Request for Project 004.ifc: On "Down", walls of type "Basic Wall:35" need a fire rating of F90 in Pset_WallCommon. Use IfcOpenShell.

First a look at what the model holds.

```python
import ifcopenshell
import ifcopenshell.util.element

model = ifcopenshell.open("Project 004.ifc")
print(model.schema)
storey = next(s for s in model.by_type("IfcBuildingStorey") if s.Name == "Down")
walls = [e for e in ifcopenshell.util.element.get_decomposition(storey) if e.is_a("IfcWall")]
seen = {}
for e in walls:
    element_type = ifcopenshell.util.element.get_type(e)
    key = (element_type.Name if element_type != e and element_type else None, ifcopenshell.util.element.get_pset(e, "Pset_WallCommon", "FireRating"))
    seen[key] = seen.get(key, 0) + 1
for (name, value), count in sorted(seen.items(), key=str):
    print(count, "x", name, "|", value)
```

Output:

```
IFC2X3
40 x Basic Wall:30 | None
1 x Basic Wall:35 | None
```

```python
import ifcopenshell
import ifcopenshell.api.pset
import ifcopenshell.util.element

model = ifcopenshell.open("Project 004.ifc")

storey = next(s for s in model.by_type("IfcBuildingStorey") if s.Name == "Down")
walls = [e for e in ifcopenshell.util.element.get_decomposition(storey) if e.is_a("IfcWall")]

count = 0
for e in walls:
    element_type = ifcopenshell.util.element.get_type(e)
    if element_type in (None, e) or element_type.Name != "Basic Wall:35":
        continue
    # add_pset returns the element's existing set when there is one.
    pset = ifcopenshell.api.pset.add_pset(model, product=e, name="Pset_WallCommon")
    ifcopenshell.api.pset.edit_pset(model, pset=pset, properties={"FireRating": "F90"})
    count += 1

print(count, "walls updated")

model.write("Project 004_edited.ifc")
```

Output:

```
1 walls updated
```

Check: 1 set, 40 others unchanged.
